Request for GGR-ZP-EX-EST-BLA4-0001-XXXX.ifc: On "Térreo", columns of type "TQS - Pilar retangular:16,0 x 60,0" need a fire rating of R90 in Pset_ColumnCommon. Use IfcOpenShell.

First a look at what the model holds.

```python
import ifcopenshell
import ifcopenshell.util.element

model = ifcopenshell.open("GGR-ZP-EX-EST-BLA4-0001-XXXX.ifc")
print(model.schema)
storey = next(s for s in model.by_type("IfcBuildingStorey") if s.Name == "Térreo")
columns = [e for e in ifcopenshell.util.element.get_decomposition(storey) if e.is_a("IfcColumn")]
seen = {}
for e in columns:
    element_type = ifcopenshell.util.element.get_type(e)
    key = (element_type.Name if element_type != e and element_type else None, ifcopenshell.util.element.get_pset(e, "Pset_ColumnCommon", "FireRating"))
    seen[key] = seen.get(key, 0) + 1
for (name, value), count in sorted(seen.items(), key=str):
    print(count, "x", name, "|", value)
```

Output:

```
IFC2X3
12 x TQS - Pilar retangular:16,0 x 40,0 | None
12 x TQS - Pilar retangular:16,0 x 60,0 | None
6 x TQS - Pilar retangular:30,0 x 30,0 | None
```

```python
import ifcopenshell
import ifcopenshell.api.pset
import ifcopenshell.util.element

model = ifcopenshell.open("GGR-ZP-EX-EST-BLA4-0001-XXXX.ifc")

storey = next(s for s in model.by_type("IfcBuildingStorey") if s.Name == "Térreo")
columns = [e for e in ifcopenshell.util.element.get_decomposition(storey) if e.is_a("IfcColumn")]

count = 0
for e in columns:
    element_type = ifcopenshell.util.element.get_type(e)
    if element_type in (None, e) or element_type.Name != "TQS - Pilar retangular:16,0 x 60,0":
        continue
    # add_pset returns the element's existing set when there is one.
    pset = ifcopenshell.api.pset.add_pset(model, product=e, name="Pset_ColumnCommon")
    ifcopenshell.api.pset.edit_pset(model, pset=pset, properties={"FireRating": "R90"})
    count += 1

print(count, "columns updated")

model.write("GGR-ZP-EX-EST-BLA4-0001-XXXX-out.ifc")
```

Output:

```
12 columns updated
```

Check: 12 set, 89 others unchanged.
